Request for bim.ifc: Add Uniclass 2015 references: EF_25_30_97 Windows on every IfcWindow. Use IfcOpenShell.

First a look at what the model holds.

```python
import ifcopenshell

model = ifcopenshell.open("bim.ifc")
print(model.schema)
print("classifications:", [c.Name for c in model.by_type("IfcClassification")])
for ifc_class in ("IfcDoor", "IfcRoof", "IfcStair", "IfcWall", "IfcWindow"):
    print(ifc_class, len(model.by_type(ifc_class)))
```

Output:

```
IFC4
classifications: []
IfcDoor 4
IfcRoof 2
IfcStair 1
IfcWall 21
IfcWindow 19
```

```python
import ifcopenshell
import ifcopenshell.api.classification

model = ifcopenshell.open("bim.ifc")

system = ifcopenshell.api.classification.add_classification(model, classification="Uniclass 2015")

codes = {
    "IfcWindow": ("EF_25_30_97", "Windows"),
}
for ifc_class, (code, name) in codes.items():
    products = model.by_type(ifc_class)
    ifcopenshell.api.classification.add_reference(
        model, products=products, classification=system, identification=code, name=name
    )
    print(code, len(products))

model.write("bim_v2.ifc")
```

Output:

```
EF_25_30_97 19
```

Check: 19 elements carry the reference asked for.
